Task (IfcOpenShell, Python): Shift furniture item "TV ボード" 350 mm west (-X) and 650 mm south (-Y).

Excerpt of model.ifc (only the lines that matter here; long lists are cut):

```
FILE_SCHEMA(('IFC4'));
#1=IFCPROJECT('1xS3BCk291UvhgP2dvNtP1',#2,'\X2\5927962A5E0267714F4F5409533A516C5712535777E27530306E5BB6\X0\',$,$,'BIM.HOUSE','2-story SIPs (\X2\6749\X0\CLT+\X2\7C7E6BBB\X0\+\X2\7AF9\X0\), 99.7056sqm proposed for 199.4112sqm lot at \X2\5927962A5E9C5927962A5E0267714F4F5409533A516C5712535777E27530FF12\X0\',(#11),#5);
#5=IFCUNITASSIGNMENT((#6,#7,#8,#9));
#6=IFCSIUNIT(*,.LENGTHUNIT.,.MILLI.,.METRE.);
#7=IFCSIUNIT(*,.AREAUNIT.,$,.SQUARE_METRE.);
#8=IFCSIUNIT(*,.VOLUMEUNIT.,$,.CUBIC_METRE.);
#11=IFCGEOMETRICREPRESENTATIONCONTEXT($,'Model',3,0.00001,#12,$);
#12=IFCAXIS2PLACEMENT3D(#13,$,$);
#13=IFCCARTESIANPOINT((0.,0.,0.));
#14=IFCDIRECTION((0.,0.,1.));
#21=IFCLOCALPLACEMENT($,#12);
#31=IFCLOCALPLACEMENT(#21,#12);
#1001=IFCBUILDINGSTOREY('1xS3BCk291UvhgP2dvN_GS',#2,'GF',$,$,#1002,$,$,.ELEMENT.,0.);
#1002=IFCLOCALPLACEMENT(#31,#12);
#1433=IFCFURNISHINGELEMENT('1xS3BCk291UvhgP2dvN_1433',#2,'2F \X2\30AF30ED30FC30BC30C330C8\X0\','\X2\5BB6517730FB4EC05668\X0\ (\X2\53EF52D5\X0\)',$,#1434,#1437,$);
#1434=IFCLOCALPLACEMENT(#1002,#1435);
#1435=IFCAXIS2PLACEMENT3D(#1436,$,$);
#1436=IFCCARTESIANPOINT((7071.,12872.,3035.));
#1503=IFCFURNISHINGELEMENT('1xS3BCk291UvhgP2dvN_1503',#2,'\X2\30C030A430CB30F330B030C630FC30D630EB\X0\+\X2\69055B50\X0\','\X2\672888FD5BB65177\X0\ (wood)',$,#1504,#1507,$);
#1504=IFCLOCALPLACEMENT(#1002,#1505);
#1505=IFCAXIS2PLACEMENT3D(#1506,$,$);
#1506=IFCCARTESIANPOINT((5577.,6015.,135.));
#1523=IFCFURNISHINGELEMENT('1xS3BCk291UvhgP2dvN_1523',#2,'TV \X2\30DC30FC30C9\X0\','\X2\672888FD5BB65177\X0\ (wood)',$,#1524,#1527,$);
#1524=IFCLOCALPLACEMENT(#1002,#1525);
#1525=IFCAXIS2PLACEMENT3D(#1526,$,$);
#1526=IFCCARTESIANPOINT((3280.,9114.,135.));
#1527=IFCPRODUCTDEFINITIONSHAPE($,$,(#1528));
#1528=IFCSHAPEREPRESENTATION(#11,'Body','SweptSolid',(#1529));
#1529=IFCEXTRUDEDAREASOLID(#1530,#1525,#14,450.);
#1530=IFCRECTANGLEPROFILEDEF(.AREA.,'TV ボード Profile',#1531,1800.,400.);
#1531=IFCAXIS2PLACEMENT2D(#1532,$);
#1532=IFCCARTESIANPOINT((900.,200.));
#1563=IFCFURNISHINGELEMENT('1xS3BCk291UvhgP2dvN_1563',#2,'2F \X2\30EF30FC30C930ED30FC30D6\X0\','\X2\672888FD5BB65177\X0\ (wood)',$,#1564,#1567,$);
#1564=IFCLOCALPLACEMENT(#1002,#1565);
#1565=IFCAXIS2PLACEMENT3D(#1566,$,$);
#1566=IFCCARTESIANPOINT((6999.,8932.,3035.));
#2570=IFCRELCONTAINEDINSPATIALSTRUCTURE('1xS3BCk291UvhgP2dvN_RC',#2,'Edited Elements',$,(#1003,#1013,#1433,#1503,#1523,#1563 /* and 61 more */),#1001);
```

```python
import ifcopenshell
import ifcopenshell.api.geometry
import ifcopenshell.util.placement
import ifcopenshell.util.unit

model = ifcopenshell.open("model.ifc")
unit_scale = ifcopenshell.util.unit.calculate_unit_scale(model)

item = model.by_id(1523)
matrix = ifcopenshell.util.placement.get_local_placement(item.ObjectPlacement)
matrix[0, 3] -= 0.35 / unit_scale
matrix[1, 3] -= 0.65 / unit_scale
ifcopenshell.api.geometry.edit_object_placement(model, product=item, matrix=matrix, is_si=False)

print(ifcopenshell.util.placement.get_local_placement(item.ObjectPlacement).round(3) + 0.0)

model.write("model_v2.ifc")
```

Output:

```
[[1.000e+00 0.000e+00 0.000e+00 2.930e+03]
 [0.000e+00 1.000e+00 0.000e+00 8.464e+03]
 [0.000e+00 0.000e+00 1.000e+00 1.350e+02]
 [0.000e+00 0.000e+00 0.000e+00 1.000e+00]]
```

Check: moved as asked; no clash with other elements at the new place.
